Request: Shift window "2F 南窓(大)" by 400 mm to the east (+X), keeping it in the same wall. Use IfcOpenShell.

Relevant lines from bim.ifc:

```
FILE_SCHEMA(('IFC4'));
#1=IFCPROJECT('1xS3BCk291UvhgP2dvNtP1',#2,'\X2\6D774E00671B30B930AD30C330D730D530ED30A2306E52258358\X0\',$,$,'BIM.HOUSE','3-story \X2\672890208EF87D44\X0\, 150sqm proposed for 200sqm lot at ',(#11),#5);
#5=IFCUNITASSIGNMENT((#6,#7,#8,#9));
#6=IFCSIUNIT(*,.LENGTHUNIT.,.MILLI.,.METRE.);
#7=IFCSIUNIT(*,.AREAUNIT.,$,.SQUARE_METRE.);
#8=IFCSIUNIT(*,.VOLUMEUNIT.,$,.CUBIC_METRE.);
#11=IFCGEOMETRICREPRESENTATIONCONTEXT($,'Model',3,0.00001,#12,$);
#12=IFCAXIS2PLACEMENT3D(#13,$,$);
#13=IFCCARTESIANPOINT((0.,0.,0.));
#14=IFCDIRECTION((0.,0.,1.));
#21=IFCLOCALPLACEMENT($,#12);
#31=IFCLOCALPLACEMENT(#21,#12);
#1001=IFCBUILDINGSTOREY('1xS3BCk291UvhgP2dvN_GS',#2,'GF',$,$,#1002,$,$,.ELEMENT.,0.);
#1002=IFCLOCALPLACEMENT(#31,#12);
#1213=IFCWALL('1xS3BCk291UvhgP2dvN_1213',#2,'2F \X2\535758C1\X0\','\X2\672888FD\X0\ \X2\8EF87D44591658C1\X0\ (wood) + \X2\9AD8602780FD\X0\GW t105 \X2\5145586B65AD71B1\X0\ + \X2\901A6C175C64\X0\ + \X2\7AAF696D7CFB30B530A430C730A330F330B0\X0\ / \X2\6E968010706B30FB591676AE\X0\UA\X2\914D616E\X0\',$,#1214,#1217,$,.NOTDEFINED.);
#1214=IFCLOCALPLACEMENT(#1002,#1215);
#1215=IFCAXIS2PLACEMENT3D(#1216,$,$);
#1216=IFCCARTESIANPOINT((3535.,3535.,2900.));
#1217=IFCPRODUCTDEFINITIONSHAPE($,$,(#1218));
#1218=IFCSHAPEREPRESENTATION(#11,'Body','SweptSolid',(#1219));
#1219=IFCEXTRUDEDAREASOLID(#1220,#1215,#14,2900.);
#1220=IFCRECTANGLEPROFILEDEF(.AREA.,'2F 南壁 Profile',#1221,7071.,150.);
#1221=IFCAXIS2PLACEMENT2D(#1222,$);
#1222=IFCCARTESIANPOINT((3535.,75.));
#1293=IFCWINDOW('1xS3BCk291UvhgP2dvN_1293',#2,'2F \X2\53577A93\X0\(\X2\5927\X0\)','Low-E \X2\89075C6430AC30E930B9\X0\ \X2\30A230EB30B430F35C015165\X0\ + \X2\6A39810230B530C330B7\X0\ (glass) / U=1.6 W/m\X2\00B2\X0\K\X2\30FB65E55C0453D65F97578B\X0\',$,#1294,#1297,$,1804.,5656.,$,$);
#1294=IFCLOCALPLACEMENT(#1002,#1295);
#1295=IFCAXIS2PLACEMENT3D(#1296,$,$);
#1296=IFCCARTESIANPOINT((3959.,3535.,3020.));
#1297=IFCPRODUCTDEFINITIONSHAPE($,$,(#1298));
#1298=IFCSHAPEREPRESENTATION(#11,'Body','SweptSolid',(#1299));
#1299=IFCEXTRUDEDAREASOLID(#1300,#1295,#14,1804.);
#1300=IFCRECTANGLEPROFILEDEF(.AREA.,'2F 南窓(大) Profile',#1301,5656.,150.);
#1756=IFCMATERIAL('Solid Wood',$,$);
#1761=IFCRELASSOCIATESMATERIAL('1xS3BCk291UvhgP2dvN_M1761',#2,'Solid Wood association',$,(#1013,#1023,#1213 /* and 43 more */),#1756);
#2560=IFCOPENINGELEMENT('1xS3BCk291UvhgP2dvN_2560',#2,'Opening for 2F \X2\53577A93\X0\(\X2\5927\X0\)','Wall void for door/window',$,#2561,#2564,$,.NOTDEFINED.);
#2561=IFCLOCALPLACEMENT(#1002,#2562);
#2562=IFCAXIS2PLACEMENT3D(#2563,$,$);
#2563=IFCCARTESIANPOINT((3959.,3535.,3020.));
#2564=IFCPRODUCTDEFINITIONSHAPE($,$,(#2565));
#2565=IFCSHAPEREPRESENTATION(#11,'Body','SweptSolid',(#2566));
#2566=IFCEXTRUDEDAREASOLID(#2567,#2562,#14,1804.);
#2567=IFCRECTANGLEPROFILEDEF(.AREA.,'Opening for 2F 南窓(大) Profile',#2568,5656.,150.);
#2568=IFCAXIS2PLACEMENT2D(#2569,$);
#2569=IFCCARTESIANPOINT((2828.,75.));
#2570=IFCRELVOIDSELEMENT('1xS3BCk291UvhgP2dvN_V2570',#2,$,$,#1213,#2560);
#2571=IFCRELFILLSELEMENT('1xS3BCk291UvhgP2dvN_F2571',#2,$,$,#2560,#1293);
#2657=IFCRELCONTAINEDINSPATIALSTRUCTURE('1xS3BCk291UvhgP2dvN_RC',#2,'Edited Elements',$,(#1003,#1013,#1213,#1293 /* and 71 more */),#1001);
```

```python
import ifcopenshell
import ifcopenshell.api.geometry
import ifcopenshell.util.placement
import ifcopenshell.util.unit

model = ifcopenshell.open("bim.ifc")
unit_scale = ifcopenshell.util.unit.calculate_unit_scale(model)

window = model.by_id(1293)
opening = window.FillsVoids[0].RelatingOpeningElement
wall = opening.VoidsElements[0].RelatingBuildingElement

wall_matrix = ifcopenshell.util.placement.get_local_placement(wall.ObjectPlacement)
shift = wall_matrix[:3, 0] * 0.4 / unit_scale
before = ifcopenshell.util.placement.get_local_placement(window.ObjectPlacement)[:3, 3].copy()

# The window is not placed relative to its opening, so move both.
for product in (opening, window):
    matrix = ifcopenshell.util.placement.get_local_placement(product.ObjectPlacement)
    matrix[:3, 3] += shift
    ifcopenshell.api.geometry.edit_object_placement(model, product=product, matrix=matrix, is_si=False)

after = ifcopenshell.util.placement.get_local_placement(window.ObjectPlacement)[:3, 3]
print("window moved by", (after - before).round(3) + 0.0)

model.write("bim_v2.ifc")
```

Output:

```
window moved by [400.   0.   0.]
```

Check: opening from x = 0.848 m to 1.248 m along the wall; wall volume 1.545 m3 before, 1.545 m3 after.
